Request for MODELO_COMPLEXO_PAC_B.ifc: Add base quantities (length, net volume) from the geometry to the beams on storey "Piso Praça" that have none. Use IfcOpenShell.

First a look at what the model holds.

```python
import ifcopenshell
import ifcopenshell.util.element
import ifcopenshell.util.unit

model = ifcopenshell.open("MODELO_COMPLEXO_PAC_B.ifc")
print(model.schema)
for unit_type in ("LENGTHUNIT", "AREAUNIT", "VOLUMEUNIT"):
    print(unit_type, ifcopenshell.util.unit.calculate_unit_scale(model, unit_type))
storey = next(s for s in model.by_type("IfcBuildingStorey") if s.Name == "Piso Praça")
beams = [e for e in ifcopenshell.util.element.get_decomposition(storey) if e.is_a("IfcBeam")]
for e in sorted(beams, key=lambda e: e.id()):
    print(e.id(), e.is_a(), e.Name, list(ifcopenshell.util.element.get_psets(e, qtos_only=True)), sep=" | ")
```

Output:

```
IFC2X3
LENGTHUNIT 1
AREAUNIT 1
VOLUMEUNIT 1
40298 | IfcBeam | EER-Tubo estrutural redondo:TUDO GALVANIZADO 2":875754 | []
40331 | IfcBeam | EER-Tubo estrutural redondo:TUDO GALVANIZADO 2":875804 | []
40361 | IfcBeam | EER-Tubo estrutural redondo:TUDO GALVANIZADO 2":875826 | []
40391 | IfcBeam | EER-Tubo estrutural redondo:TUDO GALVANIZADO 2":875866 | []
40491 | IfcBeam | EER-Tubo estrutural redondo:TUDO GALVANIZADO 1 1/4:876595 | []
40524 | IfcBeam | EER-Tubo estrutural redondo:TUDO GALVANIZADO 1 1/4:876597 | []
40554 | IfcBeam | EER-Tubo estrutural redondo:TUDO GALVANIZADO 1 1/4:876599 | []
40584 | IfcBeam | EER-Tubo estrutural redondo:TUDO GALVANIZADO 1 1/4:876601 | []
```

```python
import ifcopenshell
import ifcopenshell.api.pset
import ifcopenshell.geom
import ifcopenshell.util.element
import ifcopenshell.util.shape
import ifcopenshell.util.unit

model = ifcopenshell.open("MODELO_COMPLEXO_PAC_B.ifc")
unit_scale = ifcopenshell.util.unit.calculate_unit_scale(model)
volume_scale = ifcopenshell.util.unit.calculate_unit_scale(model, "VOLUMEUNIT")
settings = ifcopenshell.geom.settings()

storey = next(s for s in model.by_type("IfcBuildingStorey") if s.Name == "Piso Praça")
beams = [e for e in ifcopenshell.util.element.get_decomposition(storey) if e.is_a("IfcBeam")]

for e in sorted(beams, key=lambda e: e.id()):
    if ifcopenshell.util.element.get_psets(e, qtos_only=True, should_inherit=False):
        continue
    # Geometry comes back in metres, in the element's own axes.
    shape = ifcopenshell.geom.create_shape(settings, e)
    values = {
        "Length": ifcopenshell.util.shape.get_max_xyz(shape.geometry) / unit_scale,
        "NetVolume": ifcopenshell.util.shape.get_volume(shape.geometry) / volume_scale,
    }
    qto = ifcopenshell.api.pset.add_qto(model, product=e, name="BaseQuantities")
    ifcopenshell.api.pset.edit_qto(model, qto=qto, properties=values)
    print(e.id(), {k: round(v, 3) for k, v in values.items()})

model.write("MODELO_COMPLEXO_PAC_B_edited.ifc")
```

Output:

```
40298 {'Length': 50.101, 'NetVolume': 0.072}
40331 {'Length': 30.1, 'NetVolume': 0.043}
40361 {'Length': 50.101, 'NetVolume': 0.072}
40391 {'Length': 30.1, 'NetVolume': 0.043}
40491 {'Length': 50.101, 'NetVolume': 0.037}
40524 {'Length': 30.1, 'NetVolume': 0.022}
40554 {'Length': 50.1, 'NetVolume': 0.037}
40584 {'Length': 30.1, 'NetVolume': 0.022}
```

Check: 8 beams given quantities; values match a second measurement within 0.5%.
